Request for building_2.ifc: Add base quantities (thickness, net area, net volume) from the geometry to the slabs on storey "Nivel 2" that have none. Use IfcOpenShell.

First a look at what the model holds.

```python
import ifcopenshell
import ifcopenshell.util.element
import ifcopenshell.util.unit

model = ifcopenshell.open("building_2.ifc")
print(model.schema)
for unit_type in ("LENGTHUNIT", "AREAUNIT", "VOLUMEUNIT"):
    print(unit_type, ifcopenshell.util.unit.calculate_unit_scale(model, unit_type))
storey = next(s for s in model.by_type("IfcBuildingStorey") if s.Name == "Nivel 2")
slabs = [e for e in ifcopenshell.util.element.get_decomposition(storey) if e.is_a("IfcSlab")]
for e in sorted(slabs, key=lambda e: e.id()):
    print(e.id(), e.is_a(), e.Name, list(ifcopenshell.util.element.get_psets(e, qtos_only=True)), sep=" | ")
```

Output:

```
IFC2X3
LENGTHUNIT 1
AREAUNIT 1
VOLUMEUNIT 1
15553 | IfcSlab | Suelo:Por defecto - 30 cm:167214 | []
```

```python
import ifcopenshell
import ifcopenshell.api.pset
import ifcopenshell.geom
import ifcopenshell.util.element
import ifcopenshell.util.shape
import ifcopenshell.util.unit

model = ifcopenshell.open("building_2.ifc")
unit_scale = ifcopenshell.util.unit.calculate_unit_scale(model)
area_scale = ifcopenshell.util.unit.calculate_unit_scale(model, "AREAUNIT")
volume_scale = ifcopenshell.util.unit.calculate_unit_scale(model, "VOLUMEUNIT")
settings = ifcopenshell.geom.settings()

storey = next(s for s in model.by_type("IfcBuildingStorey") if s.Name == "Nivel 2")
slabs = [e for e in ifcopenshell.util.element.get_decomposition(storey) if e.is_a("IfcSlab")]

for e in sorted(slabs, key=lambda e: e.id()):
    if ifcopenshell.util.element.get_psets(e, qtos_only=True, should_inherit=False):
        continue
    # Geometry comes back in metres, in the element's own axes.
    shape = ifcopenshell.geom.create_shape(settings, e)
    values = {
        "Width": ifcopenshell.util.shape.get_z(shape.geometry) / unit_scale,
        "NetArea": ifcopenshell.util.shape.get_footprint_area(shape.geometry) / area_scale,
        "NetVolume": ifcopenshell.util.shape.get_volume(shape.geometry) / volume_scale,
    }
    qto = ifcopenshell.api.pset.add_qto(model, product=e, name="BaseQuantities")
    ifcopenshell.api.pset.edit_qto(model, qto=qto, properties=values)
    print(e.id(), {k: round(v, 3) for k, v in values.items()})

model.write("building_2_rev.ifc")
```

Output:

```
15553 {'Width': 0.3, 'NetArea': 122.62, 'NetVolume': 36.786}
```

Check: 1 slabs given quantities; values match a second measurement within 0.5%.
